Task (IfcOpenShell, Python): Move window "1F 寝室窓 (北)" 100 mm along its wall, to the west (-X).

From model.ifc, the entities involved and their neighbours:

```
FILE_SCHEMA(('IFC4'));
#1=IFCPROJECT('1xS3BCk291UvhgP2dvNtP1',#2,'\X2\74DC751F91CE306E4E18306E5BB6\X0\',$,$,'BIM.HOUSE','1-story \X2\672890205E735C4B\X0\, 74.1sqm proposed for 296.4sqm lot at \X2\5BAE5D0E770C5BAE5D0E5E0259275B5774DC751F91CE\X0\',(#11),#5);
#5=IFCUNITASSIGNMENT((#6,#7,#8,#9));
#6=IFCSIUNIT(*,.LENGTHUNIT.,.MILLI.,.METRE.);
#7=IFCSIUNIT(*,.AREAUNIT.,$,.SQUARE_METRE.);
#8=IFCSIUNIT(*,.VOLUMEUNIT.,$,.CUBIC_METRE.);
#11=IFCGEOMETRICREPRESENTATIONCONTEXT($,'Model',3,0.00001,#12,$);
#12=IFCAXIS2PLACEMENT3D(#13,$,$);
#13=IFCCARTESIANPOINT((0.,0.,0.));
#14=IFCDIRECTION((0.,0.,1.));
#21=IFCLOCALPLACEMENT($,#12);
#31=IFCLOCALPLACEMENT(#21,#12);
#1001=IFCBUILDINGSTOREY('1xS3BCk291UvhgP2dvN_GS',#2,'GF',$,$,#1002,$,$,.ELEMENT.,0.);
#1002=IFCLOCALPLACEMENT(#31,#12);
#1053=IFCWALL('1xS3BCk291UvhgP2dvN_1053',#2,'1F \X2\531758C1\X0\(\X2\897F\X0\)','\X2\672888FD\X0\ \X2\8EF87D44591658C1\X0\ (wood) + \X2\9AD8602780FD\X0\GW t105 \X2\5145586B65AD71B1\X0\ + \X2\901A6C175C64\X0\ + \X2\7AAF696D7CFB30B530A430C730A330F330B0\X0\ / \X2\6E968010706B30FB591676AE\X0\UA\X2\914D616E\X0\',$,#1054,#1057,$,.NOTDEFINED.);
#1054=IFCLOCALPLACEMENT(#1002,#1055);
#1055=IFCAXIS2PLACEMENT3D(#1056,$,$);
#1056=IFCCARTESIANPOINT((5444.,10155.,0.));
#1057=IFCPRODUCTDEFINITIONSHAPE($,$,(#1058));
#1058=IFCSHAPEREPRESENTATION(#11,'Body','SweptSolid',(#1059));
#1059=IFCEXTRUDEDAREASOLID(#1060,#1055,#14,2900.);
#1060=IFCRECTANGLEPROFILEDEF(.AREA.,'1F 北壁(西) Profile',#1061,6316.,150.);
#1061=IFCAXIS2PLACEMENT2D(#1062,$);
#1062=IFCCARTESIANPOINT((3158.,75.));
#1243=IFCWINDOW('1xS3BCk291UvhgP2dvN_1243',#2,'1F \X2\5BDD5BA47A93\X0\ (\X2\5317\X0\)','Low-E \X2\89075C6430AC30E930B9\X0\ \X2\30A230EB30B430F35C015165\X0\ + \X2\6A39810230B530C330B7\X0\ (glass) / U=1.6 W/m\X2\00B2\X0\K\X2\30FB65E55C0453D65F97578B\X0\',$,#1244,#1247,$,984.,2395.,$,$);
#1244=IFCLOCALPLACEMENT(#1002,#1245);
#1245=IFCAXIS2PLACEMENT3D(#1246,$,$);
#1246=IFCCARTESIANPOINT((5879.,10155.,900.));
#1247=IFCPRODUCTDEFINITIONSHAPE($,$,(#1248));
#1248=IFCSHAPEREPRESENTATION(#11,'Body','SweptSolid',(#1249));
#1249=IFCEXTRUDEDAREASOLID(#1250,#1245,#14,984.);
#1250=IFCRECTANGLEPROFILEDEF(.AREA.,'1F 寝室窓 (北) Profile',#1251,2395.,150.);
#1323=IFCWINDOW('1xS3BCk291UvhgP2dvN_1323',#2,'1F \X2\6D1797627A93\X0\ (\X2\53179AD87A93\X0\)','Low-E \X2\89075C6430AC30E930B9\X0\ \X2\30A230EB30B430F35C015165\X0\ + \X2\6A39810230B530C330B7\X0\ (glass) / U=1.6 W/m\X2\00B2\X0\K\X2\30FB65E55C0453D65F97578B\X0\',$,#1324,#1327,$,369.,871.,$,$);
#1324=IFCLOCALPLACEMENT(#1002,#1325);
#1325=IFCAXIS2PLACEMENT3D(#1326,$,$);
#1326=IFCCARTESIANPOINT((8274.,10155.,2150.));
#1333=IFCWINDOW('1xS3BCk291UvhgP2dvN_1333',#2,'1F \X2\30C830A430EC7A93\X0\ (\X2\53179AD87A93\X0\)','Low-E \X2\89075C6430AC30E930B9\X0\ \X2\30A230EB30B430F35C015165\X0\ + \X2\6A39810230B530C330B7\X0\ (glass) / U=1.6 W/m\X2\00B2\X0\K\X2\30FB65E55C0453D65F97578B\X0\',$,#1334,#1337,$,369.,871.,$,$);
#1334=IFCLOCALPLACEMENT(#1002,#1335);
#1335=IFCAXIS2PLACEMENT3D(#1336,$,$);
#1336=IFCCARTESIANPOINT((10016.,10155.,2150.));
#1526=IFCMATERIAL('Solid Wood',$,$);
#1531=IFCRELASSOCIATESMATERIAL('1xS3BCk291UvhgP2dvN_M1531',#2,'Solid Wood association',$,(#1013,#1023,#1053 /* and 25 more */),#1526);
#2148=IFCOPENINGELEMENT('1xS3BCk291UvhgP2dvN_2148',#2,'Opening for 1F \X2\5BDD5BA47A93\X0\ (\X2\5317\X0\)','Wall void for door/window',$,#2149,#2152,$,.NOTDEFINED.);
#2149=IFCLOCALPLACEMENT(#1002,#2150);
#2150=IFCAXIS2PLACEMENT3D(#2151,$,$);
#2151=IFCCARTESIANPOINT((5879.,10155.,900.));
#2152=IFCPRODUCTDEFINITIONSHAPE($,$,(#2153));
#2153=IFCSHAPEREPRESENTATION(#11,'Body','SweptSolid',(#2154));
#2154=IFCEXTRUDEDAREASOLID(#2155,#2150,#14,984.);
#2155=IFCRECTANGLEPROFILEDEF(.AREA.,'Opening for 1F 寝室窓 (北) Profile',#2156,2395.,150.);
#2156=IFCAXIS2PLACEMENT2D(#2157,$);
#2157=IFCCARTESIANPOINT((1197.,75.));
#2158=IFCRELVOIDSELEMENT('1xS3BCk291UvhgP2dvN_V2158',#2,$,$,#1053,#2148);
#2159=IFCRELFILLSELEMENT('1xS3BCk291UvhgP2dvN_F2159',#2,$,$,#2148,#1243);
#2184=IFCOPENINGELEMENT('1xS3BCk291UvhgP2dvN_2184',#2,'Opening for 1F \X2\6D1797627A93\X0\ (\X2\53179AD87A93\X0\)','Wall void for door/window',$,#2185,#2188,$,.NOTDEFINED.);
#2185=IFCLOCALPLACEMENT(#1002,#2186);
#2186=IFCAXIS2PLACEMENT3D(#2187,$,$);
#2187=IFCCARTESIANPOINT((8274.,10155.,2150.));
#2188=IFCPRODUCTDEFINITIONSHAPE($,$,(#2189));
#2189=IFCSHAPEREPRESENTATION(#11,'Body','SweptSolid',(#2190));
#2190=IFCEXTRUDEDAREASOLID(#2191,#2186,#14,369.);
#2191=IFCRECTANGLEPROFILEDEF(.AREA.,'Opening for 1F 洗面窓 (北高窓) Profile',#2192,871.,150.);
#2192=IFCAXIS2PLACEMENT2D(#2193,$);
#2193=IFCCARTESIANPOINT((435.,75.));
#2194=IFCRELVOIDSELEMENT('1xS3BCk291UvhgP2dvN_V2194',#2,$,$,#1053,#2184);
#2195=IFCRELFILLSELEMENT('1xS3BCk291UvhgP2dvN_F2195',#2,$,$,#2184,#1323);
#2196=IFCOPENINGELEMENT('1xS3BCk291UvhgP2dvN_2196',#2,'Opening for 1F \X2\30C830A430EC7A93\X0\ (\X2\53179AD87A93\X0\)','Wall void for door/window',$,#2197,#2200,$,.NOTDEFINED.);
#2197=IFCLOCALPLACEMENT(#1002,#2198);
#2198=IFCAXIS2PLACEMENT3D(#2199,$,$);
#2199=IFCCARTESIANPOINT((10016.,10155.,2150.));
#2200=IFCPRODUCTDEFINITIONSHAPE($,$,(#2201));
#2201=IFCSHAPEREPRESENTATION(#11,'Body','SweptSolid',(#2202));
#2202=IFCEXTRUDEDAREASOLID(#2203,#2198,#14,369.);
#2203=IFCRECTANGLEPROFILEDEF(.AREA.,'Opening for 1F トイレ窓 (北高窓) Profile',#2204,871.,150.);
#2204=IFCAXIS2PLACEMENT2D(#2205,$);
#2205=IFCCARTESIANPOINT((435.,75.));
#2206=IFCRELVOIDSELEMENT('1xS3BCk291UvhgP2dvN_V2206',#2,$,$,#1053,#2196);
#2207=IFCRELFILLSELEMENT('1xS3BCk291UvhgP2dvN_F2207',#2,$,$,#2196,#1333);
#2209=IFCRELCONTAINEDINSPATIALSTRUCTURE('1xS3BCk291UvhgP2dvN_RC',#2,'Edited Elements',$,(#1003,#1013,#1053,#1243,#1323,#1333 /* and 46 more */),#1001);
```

```python
import ifcopenshell
import ifcopenshell.api.geometry
import ifcopenshell.util.placement

model = ifcopenshell.open("model.ifc")

window = model.by_guid("1xS3BCk291UvhgP2dvN_1243")
opening = window.FillsVoids[0].RelatingOpeningElement
wall = opening.VoidsElements[0].RelatingBuildingElement

wall_matrix = ifcopenshell.util.placement.get_local_placement(wall.ObjectPlacement)
shift = wall_matrix[:3, 0] * -100.0
before = ifcopenshell.util.placement.get_local_placement(window.ObjectPlacement)[:3, 3].copy()

# The window is not placed relative to its opening, so move both.
for product in (opening, window):
    matrix = ifcopenshell.util.placement.get_local_placement(product.ObjectPlacement)
    matrix[:3, 3] += shift
    ifcopenshell.api.geometry.edit_object_placement(model, product=product, matrix=matrix, is_si=False)

after = ifcopenshell.util.placement.get_local_placement(window.ObjectPlacement)[:3, 3]
print("window moved by", (after - before).round(3) + 0.0)

model.write("model_updated.ifc")
```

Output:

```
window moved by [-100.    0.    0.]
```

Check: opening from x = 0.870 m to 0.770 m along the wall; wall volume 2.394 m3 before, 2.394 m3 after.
